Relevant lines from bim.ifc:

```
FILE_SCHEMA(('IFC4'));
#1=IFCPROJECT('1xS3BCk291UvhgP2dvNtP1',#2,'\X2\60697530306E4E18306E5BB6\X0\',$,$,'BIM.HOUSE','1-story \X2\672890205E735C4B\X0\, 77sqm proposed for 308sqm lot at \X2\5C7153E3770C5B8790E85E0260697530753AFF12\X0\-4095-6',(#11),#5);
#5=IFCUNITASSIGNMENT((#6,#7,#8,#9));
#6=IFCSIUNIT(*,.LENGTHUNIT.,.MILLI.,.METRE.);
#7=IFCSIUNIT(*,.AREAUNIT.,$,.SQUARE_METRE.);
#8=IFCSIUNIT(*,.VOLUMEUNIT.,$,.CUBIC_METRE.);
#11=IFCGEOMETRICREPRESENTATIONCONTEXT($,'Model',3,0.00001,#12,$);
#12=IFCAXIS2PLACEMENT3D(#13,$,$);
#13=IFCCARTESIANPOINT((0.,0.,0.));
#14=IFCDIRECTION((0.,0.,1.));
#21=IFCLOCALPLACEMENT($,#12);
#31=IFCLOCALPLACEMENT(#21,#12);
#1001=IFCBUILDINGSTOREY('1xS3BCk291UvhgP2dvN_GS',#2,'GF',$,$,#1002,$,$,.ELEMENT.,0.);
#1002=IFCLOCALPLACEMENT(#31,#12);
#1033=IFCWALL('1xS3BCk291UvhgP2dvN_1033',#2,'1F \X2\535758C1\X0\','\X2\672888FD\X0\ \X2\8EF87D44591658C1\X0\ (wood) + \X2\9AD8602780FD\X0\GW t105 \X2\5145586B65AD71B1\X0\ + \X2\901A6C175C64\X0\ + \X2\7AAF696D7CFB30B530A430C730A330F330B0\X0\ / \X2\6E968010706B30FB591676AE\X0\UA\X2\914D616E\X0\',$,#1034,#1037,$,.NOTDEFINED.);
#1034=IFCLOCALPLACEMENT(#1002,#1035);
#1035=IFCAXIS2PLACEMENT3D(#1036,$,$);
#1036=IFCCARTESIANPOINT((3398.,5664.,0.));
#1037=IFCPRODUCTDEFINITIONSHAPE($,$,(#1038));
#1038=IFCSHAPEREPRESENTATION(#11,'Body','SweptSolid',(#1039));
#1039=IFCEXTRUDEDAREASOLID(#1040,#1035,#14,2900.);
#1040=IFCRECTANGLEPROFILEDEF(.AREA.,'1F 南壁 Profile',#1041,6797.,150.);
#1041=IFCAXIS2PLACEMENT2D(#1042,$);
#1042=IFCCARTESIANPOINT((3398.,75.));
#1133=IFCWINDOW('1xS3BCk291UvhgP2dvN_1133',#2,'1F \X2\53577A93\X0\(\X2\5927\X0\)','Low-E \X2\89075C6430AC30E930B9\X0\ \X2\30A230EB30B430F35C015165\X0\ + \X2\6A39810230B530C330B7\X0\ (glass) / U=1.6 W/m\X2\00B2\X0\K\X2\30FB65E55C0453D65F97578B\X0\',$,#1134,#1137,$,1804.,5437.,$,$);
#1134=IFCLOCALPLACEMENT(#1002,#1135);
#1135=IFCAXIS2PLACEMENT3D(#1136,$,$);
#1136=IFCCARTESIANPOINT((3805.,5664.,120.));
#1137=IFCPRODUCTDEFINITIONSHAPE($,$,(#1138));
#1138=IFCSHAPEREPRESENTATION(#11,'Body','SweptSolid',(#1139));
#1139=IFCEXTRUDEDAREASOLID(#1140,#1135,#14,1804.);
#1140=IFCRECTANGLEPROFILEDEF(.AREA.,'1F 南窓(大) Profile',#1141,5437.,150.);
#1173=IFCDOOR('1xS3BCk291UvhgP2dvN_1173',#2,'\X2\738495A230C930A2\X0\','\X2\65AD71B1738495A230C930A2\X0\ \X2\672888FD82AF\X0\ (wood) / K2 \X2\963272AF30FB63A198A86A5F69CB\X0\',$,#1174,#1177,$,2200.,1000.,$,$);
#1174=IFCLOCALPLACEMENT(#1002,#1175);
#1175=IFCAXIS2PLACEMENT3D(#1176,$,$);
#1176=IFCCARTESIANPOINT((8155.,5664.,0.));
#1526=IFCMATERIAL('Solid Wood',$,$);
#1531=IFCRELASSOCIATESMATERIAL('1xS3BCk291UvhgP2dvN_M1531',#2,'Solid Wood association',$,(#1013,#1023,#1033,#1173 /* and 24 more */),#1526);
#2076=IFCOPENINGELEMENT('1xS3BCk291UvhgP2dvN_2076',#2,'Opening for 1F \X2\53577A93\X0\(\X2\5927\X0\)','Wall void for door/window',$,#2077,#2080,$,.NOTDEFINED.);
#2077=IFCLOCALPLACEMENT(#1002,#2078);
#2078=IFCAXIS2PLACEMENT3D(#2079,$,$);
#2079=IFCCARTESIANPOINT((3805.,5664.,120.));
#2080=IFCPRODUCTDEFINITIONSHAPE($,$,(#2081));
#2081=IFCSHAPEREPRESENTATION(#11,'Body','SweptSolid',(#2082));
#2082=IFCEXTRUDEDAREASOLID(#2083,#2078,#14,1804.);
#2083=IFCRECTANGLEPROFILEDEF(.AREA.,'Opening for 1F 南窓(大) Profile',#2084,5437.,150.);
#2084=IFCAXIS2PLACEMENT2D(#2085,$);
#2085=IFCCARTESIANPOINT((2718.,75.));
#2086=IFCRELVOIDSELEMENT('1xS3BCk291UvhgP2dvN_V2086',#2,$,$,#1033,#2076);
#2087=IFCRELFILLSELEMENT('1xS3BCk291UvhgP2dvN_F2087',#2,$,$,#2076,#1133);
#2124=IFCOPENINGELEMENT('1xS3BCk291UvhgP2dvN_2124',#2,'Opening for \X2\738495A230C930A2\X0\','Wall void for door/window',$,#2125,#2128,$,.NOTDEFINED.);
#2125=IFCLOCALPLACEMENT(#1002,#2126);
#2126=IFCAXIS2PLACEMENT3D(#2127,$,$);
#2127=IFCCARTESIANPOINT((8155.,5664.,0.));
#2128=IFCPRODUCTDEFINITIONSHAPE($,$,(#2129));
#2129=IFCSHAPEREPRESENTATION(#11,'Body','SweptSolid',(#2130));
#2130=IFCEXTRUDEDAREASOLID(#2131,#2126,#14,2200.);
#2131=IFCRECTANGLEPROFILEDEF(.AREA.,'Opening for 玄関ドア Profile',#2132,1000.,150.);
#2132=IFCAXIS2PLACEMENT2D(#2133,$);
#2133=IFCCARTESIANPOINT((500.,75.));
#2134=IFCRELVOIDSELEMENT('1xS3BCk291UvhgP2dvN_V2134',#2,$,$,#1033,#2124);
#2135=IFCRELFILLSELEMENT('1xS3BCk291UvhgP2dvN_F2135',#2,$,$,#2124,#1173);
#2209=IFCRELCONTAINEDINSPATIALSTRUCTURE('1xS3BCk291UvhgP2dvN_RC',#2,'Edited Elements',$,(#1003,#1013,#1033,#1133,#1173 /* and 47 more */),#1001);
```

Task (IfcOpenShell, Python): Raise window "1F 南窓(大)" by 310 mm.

```python
import numpy as np
import ifcopenshell
import ifcopenshell.api.geometry
import ifcopenshell.util.placement
import ifcopenshell.util.unit

model = ifcopenshell.open("bim.ifc")
unit_scale = ifcopenshell.util.unit.calculate_unit_scale(model)

window = model.by_guid("1xS3BCk291UvhgP2dvN_1133")
opening = window.FillsVoids[0].RelatingOpeningElement
dz = 0.31 / unit_scale

shift = np.array([0.0, 0.0, dz])
# The window is not placed relative to its opening, so move both.
for product in (opening, window):
    matrix = ifcopenshell.util.placement.get_local_placement(product.ObjectPlacement)
    matrix[:3, 3] += shift
    ifcopenshell.api.geometry.edit_object_placement(model, product=product, matrix=matrix, is_si=False)

print(f"moved by {dz * unit_scale:+.3f} m")

model.write("bim_rev.ifc")
```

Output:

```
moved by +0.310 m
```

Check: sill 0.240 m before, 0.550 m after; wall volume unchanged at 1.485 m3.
